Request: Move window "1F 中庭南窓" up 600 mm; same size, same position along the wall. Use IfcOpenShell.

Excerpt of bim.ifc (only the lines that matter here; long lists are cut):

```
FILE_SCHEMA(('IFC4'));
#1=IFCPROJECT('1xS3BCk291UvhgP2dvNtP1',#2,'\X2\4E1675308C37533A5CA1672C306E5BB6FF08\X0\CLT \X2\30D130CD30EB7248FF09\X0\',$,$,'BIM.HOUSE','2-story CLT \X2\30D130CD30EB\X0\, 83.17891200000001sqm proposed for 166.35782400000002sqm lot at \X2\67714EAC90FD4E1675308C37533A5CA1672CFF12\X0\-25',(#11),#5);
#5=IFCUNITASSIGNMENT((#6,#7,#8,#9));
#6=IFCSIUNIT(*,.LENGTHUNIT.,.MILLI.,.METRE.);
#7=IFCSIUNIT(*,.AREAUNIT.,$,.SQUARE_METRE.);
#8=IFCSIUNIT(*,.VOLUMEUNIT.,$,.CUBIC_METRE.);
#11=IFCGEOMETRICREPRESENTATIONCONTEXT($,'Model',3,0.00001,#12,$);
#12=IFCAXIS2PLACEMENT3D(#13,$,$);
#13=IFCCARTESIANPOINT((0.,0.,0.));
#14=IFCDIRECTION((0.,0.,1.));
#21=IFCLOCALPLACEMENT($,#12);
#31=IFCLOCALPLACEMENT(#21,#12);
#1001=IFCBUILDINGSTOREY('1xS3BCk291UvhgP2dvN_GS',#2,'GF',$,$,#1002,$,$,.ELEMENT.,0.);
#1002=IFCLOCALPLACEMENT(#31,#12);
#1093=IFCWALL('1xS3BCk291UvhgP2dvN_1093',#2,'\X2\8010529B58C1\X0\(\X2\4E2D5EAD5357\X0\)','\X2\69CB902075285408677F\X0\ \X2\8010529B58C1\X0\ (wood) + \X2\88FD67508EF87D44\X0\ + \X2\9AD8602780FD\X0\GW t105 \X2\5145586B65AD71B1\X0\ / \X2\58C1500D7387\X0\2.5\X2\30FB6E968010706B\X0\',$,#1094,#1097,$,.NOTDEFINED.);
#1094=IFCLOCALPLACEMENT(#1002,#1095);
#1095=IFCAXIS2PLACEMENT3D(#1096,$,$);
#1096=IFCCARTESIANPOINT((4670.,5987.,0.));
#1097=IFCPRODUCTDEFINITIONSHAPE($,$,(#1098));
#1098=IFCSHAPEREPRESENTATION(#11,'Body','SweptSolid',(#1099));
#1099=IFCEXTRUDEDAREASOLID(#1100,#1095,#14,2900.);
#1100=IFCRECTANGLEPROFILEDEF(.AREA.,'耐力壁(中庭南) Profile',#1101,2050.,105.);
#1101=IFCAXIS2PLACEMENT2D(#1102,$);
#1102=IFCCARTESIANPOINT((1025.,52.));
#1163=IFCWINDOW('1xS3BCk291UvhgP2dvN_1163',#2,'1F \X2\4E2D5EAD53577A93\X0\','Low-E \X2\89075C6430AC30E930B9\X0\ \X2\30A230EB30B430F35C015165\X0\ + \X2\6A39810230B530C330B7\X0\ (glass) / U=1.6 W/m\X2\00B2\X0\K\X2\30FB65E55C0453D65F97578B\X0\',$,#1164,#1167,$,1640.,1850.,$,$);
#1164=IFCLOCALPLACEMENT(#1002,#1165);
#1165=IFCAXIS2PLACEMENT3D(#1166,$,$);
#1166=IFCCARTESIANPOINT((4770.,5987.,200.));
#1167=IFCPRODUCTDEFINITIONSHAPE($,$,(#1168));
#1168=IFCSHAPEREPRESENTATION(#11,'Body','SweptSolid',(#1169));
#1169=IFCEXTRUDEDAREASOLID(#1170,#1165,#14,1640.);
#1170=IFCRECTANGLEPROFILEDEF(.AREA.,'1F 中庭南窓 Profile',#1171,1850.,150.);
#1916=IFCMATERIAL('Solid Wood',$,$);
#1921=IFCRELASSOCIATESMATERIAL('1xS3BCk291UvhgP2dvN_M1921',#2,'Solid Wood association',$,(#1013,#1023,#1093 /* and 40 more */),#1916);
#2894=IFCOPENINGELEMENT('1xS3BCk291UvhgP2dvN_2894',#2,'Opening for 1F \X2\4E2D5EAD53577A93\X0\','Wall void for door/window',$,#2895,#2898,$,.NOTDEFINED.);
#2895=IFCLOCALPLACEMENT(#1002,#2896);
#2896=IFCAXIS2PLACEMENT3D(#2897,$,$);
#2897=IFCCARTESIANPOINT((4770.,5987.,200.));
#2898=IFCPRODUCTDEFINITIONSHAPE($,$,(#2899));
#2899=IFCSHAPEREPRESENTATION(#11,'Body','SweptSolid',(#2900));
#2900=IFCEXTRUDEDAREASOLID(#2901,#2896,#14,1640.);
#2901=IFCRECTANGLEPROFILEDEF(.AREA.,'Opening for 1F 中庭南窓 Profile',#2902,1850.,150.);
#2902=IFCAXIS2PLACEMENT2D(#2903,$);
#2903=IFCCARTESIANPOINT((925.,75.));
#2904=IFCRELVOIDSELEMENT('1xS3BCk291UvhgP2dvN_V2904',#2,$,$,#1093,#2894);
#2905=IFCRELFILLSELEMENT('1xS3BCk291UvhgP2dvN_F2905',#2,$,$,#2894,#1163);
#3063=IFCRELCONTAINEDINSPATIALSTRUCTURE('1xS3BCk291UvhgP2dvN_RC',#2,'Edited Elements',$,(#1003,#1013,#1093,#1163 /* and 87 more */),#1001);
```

```python
import numpy as np
import ifcopenshell
import ifcopenshell.api.geometry
import ifcopenshell.util.placement
import ifcopenshell.util.unit

model = ifcopenshell.open("bim.ifc")
unit_scale = ifcopenshell.util.unit.calculate_unit_scale(model)

window = model.by_id(1163)
opening = window.FillsVoids[0].RelatingOpeningElement
dz = 0.6 / unit_scale

shift = np.array([0.0, 0.0, dz])
# The window is not placed relative to its opening, so move both.
for product in (opening, window):
    matrix = ifcopenshell.util.placement.get_local_placement(product.ObjectPlacement)
    matrix[:3, 3] += shift
    ifcopenshell.api.geometry.edit_object_placement(model, product=product, matrix=matrix, is_si=False)

print(f"moved by {dz * unit_scale:+.3f} m")

model.write("bim_edited.ifc")
```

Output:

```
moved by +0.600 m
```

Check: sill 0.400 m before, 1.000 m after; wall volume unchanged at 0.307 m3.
